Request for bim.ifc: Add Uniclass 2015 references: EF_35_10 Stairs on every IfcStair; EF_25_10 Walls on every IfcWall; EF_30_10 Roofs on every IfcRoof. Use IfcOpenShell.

First a look at what the model holds.

```python
import ifcopenshell

model = ifcopenshell.open("bim.ifc")
print(model.schema)
print("classifications:", [c.Name for c in model.by_type("IfcClassification")])
for ifc_class in ("IfcDoor", "IfcRoof", "IfcStair", "IfcWall", "IfcWindow"):
    print(ifc_class, len(model.by_type(ifc_class)))
```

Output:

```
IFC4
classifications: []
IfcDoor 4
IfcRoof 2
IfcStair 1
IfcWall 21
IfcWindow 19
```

```python
import ifcopenshell
import ifcopenshell.api.classification

model = ifcopenshell.open("bim.ifc")

system = ifcopenshell.api.classification.add_classification(model, classification="Uniclass 2015")

codes = {
    "IfcStair": ("EF_35_10", "Stairs"),
    "IfcWall": ("EF_25_10", "Walls"),
    "IfcRoof": ("EF_30_10", "Roofs"),
}
for ifc_class, (code, name) in codes.items():
    products = model.by_type(ifc_class)
    ifcopenshell.api.classification.add_reference(
        model, products=products, classification=system, identification=code, name=name
    )
    print(code, len(products))

model.write("bim_rev.ifc")
```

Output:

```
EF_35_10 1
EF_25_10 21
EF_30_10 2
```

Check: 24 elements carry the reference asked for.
